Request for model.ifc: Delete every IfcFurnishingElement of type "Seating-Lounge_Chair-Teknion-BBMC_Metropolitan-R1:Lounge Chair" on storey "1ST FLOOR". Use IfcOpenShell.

First a look at what the model holds.

```python
import ifcopenshell
import ifcopenshell.util.element

model = ifcopenshell.open("model.ifc")
print(model.schema)
storey = next(s for s in model.by_type("IfcBuildingStorey") if s.Name == "1ST FLOOR")
furniture = [e for e in ifcopenshell.util.element.get_decomposition(storey) if e.is_a("IfcFurnishingElement")]
seen = {}
for e in furniture:
    element_type = ifcopenshell.util.element.get_type(e)
    name = element_type.Name if element_type not in (None, e) else None
    seen[name] = seen.get(name, 0) + 1
for name, count in sorted(seen.items(), key=str):
    print(count, "x", name)
```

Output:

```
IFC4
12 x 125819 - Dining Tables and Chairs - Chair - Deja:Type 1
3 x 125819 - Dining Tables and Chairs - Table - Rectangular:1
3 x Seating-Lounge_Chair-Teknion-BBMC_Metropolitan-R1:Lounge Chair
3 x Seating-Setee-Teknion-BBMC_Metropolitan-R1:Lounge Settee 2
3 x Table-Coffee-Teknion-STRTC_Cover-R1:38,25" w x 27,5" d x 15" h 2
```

```python
import ifcopenshell
import ifcopenshell.api.root
import ifcopenshell.util.element

model = ifcopenshell.open("model.ifc")

storey = next(s for s in model.by_type("IfcBuildingStorey") if s.Name == "1ST FLOOR")
furniture = [e for e in ifcopenshell.util.element.get_decomposition(storey) if e.is_a("IfcFurnishingElement")]
targets = [e for e in furniture if (t := ifcopenshell.util.element.get_type(e)) not in (None, e) and t.Name == "Seating-Lounge_Chair-Teknion-BBMC_Metropolitan-R1:Lounge Chair"]

for e in targets:
    ifcopenshell.api.root.remove_product(model, product=e)
print(len(targets), "removed")

model.write("model_rev.ifc")
```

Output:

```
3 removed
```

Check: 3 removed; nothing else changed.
